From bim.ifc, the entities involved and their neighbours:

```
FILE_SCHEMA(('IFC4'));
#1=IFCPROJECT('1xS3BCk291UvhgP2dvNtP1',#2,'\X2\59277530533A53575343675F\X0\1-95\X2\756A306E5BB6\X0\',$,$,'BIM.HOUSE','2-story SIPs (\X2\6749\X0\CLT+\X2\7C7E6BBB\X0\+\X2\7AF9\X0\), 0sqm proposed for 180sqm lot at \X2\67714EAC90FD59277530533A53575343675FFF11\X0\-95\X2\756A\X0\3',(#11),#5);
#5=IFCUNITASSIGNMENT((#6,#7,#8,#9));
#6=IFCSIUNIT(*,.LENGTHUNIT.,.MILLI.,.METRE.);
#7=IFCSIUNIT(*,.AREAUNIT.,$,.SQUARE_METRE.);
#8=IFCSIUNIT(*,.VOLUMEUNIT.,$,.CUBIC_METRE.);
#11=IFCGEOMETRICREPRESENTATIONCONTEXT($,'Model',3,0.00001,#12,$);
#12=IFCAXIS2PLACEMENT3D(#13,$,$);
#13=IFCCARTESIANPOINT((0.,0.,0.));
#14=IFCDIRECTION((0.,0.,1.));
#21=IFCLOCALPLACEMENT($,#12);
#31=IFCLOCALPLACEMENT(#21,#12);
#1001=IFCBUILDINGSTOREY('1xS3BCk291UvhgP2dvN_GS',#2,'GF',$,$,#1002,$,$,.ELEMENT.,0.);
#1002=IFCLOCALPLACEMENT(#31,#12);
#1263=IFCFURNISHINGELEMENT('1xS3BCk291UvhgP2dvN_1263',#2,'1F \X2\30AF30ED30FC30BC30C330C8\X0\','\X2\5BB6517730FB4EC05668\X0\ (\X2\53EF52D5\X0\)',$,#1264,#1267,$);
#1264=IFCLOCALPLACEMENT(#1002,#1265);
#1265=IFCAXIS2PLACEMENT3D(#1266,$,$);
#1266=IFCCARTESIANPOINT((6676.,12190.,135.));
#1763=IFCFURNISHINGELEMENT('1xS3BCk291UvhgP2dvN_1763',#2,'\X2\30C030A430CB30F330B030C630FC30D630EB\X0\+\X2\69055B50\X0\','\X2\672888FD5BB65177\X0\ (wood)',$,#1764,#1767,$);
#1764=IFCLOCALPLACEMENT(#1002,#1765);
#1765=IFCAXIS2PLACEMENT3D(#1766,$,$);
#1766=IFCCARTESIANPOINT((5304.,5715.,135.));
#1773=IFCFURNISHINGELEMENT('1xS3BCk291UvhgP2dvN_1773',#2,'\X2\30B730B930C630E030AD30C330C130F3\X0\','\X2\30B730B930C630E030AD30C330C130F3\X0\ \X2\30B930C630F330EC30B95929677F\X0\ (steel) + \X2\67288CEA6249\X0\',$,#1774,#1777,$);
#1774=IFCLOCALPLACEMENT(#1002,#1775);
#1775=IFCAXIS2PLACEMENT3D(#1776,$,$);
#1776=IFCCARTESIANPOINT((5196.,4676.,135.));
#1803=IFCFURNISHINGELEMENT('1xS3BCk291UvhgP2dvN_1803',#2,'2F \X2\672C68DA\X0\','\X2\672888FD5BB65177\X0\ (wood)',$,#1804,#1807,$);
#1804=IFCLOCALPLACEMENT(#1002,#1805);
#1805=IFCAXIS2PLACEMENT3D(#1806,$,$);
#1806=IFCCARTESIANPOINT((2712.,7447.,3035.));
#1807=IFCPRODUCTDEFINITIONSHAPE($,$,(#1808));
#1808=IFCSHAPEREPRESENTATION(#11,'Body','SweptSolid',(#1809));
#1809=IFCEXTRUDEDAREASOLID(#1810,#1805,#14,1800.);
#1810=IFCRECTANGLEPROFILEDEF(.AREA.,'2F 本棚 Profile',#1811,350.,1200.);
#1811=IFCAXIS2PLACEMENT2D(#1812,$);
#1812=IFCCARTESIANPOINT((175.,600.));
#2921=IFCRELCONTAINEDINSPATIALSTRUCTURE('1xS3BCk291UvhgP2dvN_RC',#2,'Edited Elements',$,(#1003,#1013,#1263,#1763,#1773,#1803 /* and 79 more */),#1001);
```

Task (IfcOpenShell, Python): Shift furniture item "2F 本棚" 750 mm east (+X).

```python
import ifcopenshell
import ifcopenshell.api.geometry
import ifcopenshell.util.placement
import ifcopenshell.util.unit

model = ifcopenshell.open("bim.ifc")
unit_scale = ifcopenshell.util.unit.calculate_unit_scale(model)

item = model.by_guid("1xS3BCk291UvhgP2dvN_1803")
matrix = ifcopenshell.util.placement.get_local_placement(item.ObjectPlacement)
matrix[0, 3] += 0.75 / unit_scale
ifcopenshell.api.geometry.edit_object_placement(model, product=item, matrix=matrix, is_si=False)

print(ifcopenshell.util.placement.get_local_placement(item.ObjectPlacement).round(3) + 0.0)

model.write("bim_edited.ifc")
```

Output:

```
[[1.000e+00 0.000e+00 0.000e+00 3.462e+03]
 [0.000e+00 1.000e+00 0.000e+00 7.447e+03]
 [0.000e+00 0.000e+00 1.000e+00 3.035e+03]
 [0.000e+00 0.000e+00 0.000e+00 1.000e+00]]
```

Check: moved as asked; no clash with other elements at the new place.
